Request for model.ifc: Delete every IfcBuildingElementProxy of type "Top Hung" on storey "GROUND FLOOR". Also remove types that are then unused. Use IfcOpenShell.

First a look at what the model holds.

```python
import ifcopenshell
import ifcopenshell.util.element

model = ifcopenshell.open("model.ifc")
print(model.schema)
storey = next(s for s in model.by_type("IfcBuildingStorey") if s.Name == "GROUND FLOOR")
proxies = [e for e in ifcopenshell.util.element.get_decomposition(storey) if e.is_a("IfcBuildingElementProxy")]
seen = {}
for e in proxies:
    element_type = ifcopenshell.util.element.get_type(e)
    name = element_type.Name if element_type not in (None, e) else None
    seen[name] = seen.get(name, 0) + 1
for name, count in sorted(seen.items(), key=str):
    print(count, "x", name)
```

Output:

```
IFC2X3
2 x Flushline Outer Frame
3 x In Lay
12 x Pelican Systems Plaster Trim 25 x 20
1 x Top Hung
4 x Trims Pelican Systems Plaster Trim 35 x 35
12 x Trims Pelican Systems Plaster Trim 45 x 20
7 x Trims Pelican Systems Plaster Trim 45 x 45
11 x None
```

```python
import ifcopenshell
import ifcopenshell.api.root
import ifcopenshell.util.element

model = ifcopenshell.open("model.ifc")

storey = next(s for s in model.by_type("IfcBuildingStorey") if s.Name == "GROUND FLOOR")
proxies = [e for e in ifcopenshell.util.element.get_decomposition(storey) if e.is_a("IfcBuildingElementProxy")]
targets = [e for e in proxies if (t := ifcopenshell.util.element.get_type(e)) not in (None, e) and t.Name == "Top Hung"]
types = {ifcopenshell.util.element.get_type(e) for e in targets} - {None, *targets}

for e in targets:
    ifcopenshell.api.root.remove_product(model, product=e)
print(len(targets), "removed")

unused = [t for t in types if not ifcopenshell.util.element.get_types(t)]
for t in unused:
    ifcopenshell.api.root.remove_product(model, product=t)
print(len(unused), "unused types removed")

model.write("model_v2.ifc")
```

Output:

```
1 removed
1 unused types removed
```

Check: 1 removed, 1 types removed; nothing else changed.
